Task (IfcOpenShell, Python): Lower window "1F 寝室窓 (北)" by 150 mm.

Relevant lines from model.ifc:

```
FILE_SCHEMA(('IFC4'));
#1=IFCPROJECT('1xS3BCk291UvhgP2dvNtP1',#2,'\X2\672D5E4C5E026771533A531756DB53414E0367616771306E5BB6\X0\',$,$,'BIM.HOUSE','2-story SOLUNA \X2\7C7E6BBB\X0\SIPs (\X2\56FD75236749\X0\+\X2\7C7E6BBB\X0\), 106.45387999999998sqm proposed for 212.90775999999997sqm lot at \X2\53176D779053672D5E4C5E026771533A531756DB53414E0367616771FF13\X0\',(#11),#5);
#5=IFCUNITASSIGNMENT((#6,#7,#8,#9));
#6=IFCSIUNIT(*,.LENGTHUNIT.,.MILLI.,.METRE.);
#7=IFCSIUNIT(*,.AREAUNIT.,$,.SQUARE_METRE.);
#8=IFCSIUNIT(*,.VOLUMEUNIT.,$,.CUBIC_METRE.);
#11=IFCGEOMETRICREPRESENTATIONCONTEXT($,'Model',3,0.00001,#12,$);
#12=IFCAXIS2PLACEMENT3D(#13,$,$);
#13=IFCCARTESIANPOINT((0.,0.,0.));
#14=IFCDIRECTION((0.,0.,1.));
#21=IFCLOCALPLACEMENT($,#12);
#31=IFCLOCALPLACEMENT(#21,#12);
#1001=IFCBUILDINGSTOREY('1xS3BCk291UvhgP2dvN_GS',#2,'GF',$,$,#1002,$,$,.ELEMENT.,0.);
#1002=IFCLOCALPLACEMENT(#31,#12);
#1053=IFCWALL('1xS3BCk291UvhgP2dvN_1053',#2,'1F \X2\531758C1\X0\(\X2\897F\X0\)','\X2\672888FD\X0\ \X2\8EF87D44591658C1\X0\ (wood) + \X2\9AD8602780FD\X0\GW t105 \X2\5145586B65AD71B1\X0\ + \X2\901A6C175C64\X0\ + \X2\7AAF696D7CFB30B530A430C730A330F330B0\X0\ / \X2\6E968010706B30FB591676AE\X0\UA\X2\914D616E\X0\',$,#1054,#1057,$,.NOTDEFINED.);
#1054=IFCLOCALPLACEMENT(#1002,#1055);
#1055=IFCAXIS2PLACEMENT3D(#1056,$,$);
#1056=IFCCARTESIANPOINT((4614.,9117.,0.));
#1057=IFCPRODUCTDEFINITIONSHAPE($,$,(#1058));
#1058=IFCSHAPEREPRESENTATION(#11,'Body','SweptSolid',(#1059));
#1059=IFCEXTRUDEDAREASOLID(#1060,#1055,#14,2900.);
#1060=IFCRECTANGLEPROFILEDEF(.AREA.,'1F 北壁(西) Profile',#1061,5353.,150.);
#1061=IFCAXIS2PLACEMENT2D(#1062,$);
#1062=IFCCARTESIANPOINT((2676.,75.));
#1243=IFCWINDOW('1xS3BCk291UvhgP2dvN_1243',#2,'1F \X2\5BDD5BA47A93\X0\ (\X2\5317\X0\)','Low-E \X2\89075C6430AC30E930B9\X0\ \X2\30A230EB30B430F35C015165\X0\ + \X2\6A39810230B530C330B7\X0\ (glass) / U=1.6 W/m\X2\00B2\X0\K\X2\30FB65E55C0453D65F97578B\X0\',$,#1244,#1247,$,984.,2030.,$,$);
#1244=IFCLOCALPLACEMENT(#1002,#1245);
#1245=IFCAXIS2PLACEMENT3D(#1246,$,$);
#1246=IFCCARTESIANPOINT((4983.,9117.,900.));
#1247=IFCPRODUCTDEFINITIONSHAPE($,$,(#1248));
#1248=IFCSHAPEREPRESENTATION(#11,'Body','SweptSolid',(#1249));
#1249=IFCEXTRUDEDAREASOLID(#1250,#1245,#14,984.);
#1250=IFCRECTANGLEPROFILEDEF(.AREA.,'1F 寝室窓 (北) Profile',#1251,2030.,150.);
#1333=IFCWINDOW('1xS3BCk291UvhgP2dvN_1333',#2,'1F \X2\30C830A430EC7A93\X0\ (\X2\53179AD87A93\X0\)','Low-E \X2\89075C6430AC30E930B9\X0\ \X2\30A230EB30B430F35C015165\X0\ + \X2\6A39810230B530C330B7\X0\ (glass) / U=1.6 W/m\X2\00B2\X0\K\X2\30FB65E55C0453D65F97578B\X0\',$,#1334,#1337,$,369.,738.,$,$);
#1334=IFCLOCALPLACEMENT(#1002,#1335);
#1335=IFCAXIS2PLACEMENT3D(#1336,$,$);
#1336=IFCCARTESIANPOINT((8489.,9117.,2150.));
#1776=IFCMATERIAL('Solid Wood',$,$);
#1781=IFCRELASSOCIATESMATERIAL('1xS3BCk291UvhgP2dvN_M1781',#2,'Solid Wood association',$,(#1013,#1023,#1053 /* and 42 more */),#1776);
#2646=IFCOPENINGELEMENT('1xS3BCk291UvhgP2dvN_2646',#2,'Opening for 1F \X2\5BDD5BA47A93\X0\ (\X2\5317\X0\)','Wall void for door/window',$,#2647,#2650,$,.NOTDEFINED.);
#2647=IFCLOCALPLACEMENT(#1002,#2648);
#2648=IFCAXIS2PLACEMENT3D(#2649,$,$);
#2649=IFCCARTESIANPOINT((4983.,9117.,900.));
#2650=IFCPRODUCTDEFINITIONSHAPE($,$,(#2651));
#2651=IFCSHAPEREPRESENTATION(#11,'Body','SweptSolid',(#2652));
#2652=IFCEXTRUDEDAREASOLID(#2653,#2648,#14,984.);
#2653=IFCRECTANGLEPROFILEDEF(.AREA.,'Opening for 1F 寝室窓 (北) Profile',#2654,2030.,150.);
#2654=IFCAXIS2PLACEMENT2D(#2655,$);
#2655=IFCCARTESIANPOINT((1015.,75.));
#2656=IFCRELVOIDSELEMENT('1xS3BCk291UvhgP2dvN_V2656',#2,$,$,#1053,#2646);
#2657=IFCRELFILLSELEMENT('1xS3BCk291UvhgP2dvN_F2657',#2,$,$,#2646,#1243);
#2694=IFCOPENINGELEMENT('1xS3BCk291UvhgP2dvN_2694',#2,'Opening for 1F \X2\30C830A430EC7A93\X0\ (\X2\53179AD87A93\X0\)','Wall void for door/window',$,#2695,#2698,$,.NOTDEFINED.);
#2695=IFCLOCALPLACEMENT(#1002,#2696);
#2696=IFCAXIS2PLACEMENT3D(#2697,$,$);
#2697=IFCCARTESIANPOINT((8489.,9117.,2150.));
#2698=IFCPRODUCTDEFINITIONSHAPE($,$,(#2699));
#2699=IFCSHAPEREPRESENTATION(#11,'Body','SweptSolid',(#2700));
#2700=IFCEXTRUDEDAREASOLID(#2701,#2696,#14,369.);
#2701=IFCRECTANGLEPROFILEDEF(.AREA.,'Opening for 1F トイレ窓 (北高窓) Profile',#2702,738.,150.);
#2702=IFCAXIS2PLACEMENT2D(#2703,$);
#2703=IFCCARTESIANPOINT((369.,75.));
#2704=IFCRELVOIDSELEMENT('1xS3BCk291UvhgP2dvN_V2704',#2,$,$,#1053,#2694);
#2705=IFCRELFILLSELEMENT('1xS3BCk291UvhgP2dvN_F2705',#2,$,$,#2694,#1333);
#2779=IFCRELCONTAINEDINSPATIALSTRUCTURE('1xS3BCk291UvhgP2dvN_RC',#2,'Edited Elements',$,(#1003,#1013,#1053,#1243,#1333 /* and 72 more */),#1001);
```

```python
import numpy as np
import ifcopenshell
import ifcopenshell.api.geometry
import ifcopenshell.util.placement
import ifcopenshell.util.unit

model = ifcopenshell.open("model.ifc")
unit_scale = ifcopenshell.util.unit.calculate_unit_scale(model)

window = model.by_guid("1xS3BCk291UvhgP2dvN_1243")
opening = window.FillsVoids[0].RelatingOpeningElement
dz = -0.15 / unit_scale

shift = np.array([0.0, 0.0, dz])
# The window is not placed relative to its opening, so move both.
for product in (opening, window):
    matrix = ifcopenshell.util.placement.get_local_placement(product.ObjectPlacement)
    matrix[:3, 3] += shift
    ifcopenshell.api.geometry.edit_object_placement(model, product=product, matrix=matrix, is_si=False)

print(f"moved by {dz * unit_scale:+.3f} m")

model.write("model_edited.ifc")
```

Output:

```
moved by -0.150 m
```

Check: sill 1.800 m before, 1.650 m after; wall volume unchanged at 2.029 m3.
